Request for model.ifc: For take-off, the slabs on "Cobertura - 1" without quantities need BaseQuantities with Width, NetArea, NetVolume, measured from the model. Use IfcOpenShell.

First a look at what the model holds.

```python
import ifcopenshell
import ifcopenshell.util.element
import ifcopenshell.util.unit

model = ifcopenshell.open("model.ifc")
print(model.schema)
for unit_type in ("LENGTHUNIT", "AREAUNIT", "VOLUMEUNIT"):
    print(unit_type, ifcopenshell.util.unit.calculate_unit_scale(model, unit_type))
storey = next(s for s in model.by_type("IfcBuildingStorey") if s.Name == "Cobertura - 1")
slabs = [e for e in ifcopenshell.util.element.get_decomposition(storey) if e.is_a("IfcSlab")]
for e in sorted(slabs, key=lambda e: e.id()):
    print(e.id(), e.is_a(), e.Name, list(ifcopenshell.util.element.get_psets(e, qtos_only=True)), sep=" | ")
```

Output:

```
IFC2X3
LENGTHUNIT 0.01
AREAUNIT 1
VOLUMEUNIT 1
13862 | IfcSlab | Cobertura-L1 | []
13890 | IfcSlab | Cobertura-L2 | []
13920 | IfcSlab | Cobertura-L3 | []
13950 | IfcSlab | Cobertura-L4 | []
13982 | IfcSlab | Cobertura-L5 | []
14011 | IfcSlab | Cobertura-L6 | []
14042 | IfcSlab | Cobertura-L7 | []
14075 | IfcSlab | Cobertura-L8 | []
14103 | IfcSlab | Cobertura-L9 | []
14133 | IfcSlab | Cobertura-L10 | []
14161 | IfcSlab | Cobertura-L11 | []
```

```python
import ifcopenshell
import ifcopenshell.api.pset
import ifcopenshell.geom
import ifcopenshell.util.element
import ifcopenshell.util.shape
import ifcopenshell.util.unit

model = ifcopenshell.open("model.ifc")
unit_scale = ifcopenshell.util.unit.calculate_unit_scale(model)
area_scale = ifcopenshell.util.unit.calculate_unit_scale(model, "AREAUNIT")
volume_scale = ifcopenshell.util.unit.calculate_unit_scale(model, "VOLUMEUNIT")
settings = ifcopenshell.geom.settings()

storey = next(s for s in model.by_type("IfcBuildingStorey") if s.Name == "Cobertura - 1")
slabs = [e for e in ifcopenshell.util.element.get_decomposition(storey) if e.is_a("IfcSlab")]

for e in sorted(slabs, key=lambda e: e.id()):
    if ifcopenshell.util.element.get_psets(e, qtos_only=True, should_inherit=False):
        continue
    # Geometry comes back in metres, in the element's own axes.
    shape = ifcopenshell.geom.create_shape(settings, e)
    values = {
        "Width": ifcopenshell.util.shape.get_z(shape.geometry) / unit_scale,
        "NetArea": ifcopenshell.util.shape.get_footprint_area(shape.geometry) / area_scale,
        "NetVolume": ifcopenshell.util.shape.get_volume(shape.geometry) / volume_scale,
    }
    qto = ifcopenshell.api.pset.add_qto(model, product=e, name="BaseQuantities")
    ifcopenshell.api.pset.edit_qto(model, qto=qto, properties=values)
    print(e.id(), {k: round(v, 3) for k, v in values.items()})

model.write("model_rev.ifc")
```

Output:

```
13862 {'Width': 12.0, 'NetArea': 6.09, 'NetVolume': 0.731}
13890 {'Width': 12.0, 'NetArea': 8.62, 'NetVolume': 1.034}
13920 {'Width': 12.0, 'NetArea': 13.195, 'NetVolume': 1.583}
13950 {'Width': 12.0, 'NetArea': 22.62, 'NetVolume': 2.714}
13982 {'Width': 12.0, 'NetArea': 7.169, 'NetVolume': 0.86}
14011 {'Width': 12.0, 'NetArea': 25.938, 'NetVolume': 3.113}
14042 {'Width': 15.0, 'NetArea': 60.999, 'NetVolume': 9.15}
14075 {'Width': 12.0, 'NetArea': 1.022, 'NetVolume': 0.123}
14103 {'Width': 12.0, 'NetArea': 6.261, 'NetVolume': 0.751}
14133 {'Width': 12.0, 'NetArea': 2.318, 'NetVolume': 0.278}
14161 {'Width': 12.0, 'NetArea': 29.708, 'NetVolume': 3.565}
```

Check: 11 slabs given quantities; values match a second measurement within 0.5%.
